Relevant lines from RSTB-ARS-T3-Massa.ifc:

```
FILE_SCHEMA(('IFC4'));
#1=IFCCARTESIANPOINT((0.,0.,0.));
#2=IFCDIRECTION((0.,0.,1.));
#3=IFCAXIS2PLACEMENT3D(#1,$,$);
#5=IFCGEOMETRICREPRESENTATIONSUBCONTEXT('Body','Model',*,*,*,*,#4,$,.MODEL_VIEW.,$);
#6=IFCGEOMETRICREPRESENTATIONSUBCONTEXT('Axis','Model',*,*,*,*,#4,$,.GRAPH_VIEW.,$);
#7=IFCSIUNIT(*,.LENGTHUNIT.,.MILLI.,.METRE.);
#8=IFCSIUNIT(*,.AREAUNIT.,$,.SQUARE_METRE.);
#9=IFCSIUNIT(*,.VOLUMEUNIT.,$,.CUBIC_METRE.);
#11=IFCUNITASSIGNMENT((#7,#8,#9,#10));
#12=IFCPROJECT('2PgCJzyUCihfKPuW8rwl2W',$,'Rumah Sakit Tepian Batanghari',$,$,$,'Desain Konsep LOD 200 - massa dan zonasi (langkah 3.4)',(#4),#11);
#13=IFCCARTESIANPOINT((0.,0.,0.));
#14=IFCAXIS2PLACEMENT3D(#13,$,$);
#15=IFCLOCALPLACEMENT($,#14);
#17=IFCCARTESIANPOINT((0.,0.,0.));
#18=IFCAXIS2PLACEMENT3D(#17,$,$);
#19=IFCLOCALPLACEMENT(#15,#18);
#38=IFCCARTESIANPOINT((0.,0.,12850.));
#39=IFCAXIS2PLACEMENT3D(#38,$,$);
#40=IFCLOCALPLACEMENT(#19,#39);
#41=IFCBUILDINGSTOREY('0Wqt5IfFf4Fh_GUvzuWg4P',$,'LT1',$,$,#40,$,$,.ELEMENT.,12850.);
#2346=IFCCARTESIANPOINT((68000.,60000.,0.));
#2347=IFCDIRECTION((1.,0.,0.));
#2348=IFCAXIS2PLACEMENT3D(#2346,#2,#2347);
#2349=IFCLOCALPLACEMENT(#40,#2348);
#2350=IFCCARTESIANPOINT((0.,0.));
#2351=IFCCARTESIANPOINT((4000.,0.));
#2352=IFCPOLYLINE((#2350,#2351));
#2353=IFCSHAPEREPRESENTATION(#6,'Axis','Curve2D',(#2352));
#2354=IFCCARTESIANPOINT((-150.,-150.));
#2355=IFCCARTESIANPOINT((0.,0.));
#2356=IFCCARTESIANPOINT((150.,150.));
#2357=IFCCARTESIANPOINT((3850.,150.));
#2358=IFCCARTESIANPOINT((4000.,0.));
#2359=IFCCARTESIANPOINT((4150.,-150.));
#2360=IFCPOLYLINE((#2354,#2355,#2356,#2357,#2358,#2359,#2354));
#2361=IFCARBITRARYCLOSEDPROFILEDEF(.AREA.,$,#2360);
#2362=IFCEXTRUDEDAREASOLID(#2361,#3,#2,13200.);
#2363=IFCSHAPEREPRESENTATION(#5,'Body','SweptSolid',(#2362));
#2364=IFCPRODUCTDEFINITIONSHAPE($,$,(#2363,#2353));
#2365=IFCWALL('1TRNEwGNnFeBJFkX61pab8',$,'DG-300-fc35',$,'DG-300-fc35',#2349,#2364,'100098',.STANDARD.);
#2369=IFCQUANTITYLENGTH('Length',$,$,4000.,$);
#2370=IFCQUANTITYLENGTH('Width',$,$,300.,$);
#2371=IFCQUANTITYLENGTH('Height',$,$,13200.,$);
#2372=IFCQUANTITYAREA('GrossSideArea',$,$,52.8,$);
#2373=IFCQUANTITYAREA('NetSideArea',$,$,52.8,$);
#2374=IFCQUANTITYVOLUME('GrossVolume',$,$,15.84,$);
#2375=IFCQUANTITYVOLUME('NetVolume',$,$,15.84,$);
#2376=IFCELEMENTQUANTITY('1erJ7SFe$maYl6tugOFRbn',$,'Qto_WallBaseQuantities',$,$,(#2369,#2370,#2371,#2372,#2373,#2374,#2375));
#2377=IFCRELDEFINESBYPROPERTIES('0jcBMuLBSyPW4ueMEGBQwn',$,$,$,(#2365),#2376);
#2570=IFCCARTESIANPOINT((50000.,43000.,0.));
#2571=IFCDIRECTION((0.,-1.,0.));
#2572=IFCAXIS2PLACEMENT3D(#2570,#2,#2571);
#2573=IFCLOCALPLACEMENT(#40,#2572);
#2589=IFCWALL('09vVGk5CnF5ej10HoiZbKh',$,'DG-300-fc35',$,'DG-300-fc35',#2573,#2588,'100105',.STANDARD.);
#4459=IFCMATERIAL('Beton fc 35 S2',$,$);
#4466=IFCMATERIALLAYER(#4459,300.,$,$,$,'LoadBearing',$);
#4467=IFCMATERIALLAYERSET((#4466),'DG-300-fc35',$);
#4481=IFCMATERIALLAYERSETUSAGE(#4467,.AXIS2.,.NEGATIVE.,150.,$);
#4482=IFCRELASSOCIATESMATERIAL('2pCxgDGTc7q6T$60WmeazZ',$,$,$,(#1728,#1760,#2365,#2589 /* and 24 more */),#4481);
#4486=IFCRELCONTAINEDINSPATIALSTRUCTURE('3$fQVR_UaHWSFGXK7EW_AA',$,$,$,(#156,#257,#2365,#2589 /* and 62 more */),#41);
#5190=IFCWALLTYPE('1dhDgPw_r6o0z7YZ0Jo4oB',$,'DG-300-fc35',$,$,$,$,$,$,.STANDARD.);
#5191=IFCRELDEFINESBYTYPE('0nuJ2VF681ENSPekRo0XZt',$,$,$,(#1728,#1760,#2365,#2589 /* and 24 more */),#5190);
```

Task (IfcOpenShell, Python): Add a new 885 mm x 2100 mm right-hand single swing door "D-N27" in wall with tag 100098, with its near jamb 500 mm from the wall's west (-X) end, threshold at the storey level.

```python
import numpy as np
import ifcopenshell
import ifcopenshell.api.feature
import ifcopenshell.api.geometry
import ifcopenshell.api.pset
import ifcopenshell.api.root
import ifcopenshell.api.spatial
import ifcopenshell.geom
import ifcopenshell.util.element
import ifcopenshell.util.placement
import ifcopenshell.util.representation
import ifcopenshell.util.shape
import ifcopenshell.util.unit

model = ifcopenshell.open("RSTB-ARS-T3-Massa.ifc")
unit_scale = ifcopenshell.util.unit.calculate_unit_scale(model)
area_scale = ifcopenshell.util.unit.calculate_unit_scale(model, "AREAUNIT")
volume_scale = ifcopenshell.util.unit.calculate_unit_scale(model, "VOLUMEUNIT")
settings = ifcopenshell.geom.settings()


def volume(element):
    """Net volume in cubic metres, openings subtracted."""
    shape = ifcopenshell.geom.create_shape(settings, element)
    return ifcopenshell.util.shape.get_volume(shape.geometry)


wall = model.by_guid("1TRNEwGNnFeBJFkX61pab8")
storey = ifcopenshell.util.element.get_container(wall, ifc_class="IfcBuildingStorey")
context = ifcopenshell.util.representation.get_context(model, "Model", "Body", "MODEL_VIEW")
before = volume(wall)

width, height, from_end, sill = 0.885, 2.1, 0.5, 0.0  # metres

# The wall runs along its own X axis, and the end named is its -X end.
wall_shape = ifcopenshell.geom.create_shape(settings, wall)
x, y, z = ifcopenshell.util.shape.get_vertices(wall_shape.geometry).T
start = x.min() + from_end
face, thickness = float(y.min()), float(y.max() - y.min())
wall_matrix = ifcopenshell.util.placement.get_local_placement(wall.ObjectPlacement)
level = ifcopenshell.util.placement.get_local_placement(storey.ObjectPlacement)[2, 3]


def in_wall(x, y):
    """Placement at x, y metres in the wall's axes, at sill height."""
    matrix = wall_matrix.copy()
    matrix[:, 3] = wall_matrix @ np.array([x / unit_scale, y / unit_scale, 0.0, 1.0])
    matrix[2, 3] = level + sill / unit_scale
    return matrix


# Opening: a box that overshoots both wall faces by 50 mm.
opening = ifcopenshell.api.root.create_entity(model, ifc_class="IfcOpeningElement", predefined_type="OPENING")
box = ifcopenshell.api.geometry.add_wall_representation(
    model, context=context, length=width, height=height, thickness=thickness + 0.1
)
ifcopenshell.api.geometry.assign_representation(model, product=opening, representation=box)
ifcopenshell.api.geometry.edit_object_placement(model, product=opening, matrix=in_wall(start, face - 0.05), is_si=False)
ifcopenshell.api.feature.add_feature(model, feature=opening, element=wall)

door = ifcopenshell.api.root.create_entity(model, ifc_class="IfcDoor", name="D-N27", predefined_type="DOOR")
door.OverallWidth, door.OverallHeight = width / unit_scale, height / unit_scale
door.OperationType = "SINGLE_SWING_RIGHT"
body = ifcopenshell.api.geometry.add_door_representation(
    model,
    context=context,
    overall_width=door.OverallWidth,
    overall_height=door.OverallHeight,
    operation_type="SINGLE_SWING_RIGHT",
    lining_properties={"LiningDepth": thickness / unit_scale, "ThresholdDepth": thickness / unit_scale},
)
ifcopenshell.api.geometry.assign_representation(model, product=door, representation=body)
ifcopenshell.api.spatial.assign_container(model, products=[door], relating_structure=storey)
ifcopenshell.api.feature.add_filling(model, opening=opening, element=door)

# The lining spans the wall, so the door starts at the wall face.
ifcopenshell.api.geometry.edit_object_placement(model, product=door, matrix=in_wall(start, face), is_si=False)

after = volume(wall)

# Update the wall's stored quantities.
qto = model.by_id(ifcopenshell.util.element.get_pset(wall, "Qto_WallBaseQuantities", should_inherit=False)["id"])
ifcopenshell.api.pset.edit_qto(model, qto=qto, properties={
    "NetSideArea": after / thickness / area_scale,
    "NetVolume": after / volume_scale,
})

print(f"wall volume {before:.3f} -> {after:.3f} m3")

model.write("RSTB-ARS-T3-Massa_v2.ifc")
```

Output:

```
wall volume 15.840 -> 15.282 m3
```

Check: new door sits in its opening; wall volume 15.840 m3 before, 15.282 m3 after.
